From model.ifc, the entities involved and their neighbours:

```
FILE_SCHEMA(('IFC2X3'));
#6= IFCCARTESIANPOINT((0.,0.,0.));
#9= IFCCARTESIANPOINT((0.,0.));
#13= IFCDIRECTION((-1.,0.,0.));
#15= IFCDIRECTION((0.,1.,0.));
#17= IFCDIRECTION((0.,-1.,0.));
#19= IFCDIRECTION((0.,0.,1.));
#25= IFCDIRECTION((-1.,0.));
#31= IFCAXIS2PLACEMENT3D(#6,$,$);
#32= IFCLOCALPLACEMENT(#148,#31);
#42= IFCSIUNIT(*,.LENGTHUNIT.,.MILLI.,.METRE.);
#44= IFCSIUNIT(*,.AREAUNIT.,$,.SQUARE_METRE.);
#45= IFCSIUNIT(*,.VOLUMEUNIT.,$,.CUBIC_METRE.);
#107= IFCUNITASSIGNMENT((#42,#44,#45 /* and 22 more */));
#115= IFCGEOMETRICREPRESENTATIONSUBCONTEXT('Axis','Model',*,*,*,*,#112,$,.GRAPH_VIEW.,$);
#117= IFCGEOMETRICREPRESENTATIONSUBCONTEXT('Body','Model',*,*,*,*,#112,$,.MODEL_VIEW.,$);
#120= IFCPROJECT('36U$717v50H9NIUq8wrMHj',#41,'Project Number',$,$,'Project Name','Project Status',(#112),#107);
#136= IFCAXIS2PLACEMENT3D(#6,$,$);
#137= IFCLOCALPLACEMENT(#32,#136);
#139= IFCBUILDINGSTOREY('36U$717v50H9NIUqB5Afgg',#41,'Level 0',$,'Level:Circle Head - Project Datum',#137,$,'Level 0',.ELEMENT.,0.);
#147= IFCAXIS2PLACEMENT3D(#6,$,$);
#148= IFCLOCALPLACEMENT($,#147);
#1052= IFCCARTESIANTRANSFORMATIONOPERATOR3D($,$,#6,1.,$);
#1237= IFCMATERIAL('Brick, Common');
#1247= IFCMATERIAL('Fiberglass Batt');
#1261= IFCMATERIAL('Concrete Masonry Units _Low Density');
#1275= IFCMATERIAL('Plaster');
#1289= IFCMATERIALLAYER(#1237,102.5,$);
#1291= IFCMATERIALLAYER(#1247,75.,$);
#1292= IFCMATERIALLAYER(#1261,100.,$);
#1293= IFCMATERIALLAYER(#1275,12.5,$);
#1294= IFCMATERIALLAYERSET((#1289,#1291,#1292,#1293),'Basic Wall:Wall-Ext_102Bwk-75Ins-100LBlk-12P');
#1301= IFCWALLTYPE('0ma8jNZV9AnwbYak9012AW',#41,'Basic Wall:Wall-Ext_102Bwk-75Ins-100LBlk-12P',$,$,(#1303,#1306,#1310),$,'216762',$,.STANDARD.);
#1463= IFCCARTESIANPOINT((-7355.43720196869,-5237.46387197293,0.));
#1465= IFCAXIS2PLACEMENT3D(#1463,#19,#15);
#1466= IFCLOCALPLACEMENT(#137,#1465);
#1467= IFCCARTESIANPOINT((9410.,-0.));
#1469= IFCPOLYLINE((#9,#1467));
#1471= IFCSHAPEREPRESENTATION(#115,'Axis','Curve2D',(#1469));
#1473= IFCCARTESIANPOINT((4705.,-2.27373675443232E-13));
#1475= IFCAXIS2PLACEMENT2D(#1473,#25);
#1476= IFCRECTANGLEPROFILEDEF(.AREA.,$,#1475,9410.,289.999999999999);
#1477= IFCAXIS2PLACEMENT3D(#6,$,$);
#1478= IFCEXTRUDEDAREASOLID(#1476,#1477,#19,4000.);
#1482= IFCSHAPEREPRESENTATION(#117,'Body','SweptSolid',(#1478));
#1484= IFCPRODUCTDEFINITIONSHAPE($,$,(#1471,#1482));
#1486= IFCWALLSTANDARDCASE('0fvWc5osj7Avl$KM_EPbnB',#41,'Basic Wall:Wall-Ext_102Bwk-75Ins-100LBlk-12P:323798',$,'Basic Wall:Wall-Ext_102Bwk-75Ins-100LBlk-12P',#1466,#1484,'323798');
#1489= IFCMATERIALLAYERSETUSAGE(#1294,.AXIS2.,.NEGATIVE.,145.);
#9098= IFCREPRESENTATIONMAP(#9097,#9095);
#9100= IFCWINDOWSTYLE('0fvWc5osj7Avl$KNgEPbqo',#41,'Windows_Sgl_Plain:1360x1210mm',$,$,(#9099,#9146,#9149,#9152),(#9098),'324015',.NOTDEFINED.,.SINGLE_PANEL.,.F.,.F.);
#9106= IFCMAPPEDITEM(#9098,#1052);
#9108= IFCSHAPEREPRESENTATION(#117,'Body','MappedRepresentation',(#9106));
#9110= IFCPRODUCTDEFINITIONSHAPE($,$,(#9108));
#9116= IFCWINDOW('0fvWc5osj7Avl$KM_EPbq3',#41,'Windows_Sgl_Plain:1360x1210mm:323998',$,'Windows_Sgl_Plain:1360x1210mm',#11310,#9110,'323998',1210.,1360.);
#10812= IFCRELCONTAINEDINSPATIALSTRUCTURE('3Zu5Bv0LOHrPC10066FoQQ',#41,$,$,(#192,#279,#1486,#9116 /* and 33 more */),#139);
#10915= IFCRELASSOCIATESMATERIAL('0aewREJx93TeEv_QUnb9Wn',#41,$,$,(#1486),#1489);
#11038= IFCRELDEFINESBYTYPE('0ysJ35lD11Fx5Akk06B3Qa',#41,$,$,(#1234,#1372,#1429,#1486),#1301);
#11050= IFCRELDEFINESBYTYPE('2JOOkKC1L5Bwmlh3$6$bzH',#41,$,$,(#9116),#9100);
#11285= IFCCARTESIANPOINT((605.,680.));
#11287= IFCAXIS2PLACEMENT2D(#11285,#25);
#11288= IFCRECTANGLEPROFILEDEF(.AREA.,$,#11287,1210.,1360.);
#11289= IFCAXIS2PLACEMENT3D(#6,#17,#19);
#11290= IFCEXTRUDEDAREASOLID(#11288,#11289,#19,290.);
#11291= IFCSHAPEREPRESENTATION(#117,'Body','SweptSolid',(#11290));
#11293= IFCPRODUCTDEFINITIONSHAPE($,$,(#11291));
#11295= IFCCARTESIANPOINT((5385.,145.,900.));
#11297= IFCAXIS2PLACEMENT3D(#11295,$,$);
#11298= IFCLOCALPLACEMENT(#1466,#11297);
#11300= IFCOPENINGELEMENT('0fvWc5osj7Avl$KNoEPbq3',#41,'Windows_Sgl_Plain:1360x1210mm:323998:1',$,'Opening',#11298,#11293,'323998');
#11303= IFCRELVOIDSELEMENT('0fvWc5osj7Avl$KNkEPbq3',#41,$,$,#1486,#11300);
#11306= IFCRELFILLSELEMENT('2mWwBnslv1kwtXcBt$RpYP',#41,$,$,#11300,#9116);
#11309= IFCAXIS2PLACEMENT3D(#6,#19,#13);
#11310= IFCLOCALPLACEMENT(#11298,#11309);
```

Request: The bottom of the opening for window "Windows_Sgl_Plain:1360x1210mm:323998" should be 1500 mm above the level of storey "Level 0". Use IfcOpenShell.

```python
import numpy as np
import ifcopenshell
import ifcopenshell.api.geometry
import ifcopenshell.geom
import ifcopenshell.util.element
import ifcopenshell.util.placement
import ifcopenshell.util.shape
import ifcopenshell.util.unit

model = ifcopenshell.open("model.ifc")
unit_scale = ifcopenshell.util.unit.calculate_unit_scale(model)

window = model.by_id(9116)
opening = window.FillsVoids[0].RelatingOpeningElement
storey = ifcopenshell.util.element.get_container(window, ifc_class="IfcBuildingStorey")
level = ifcopenshell.util.placement.get_local_placement(storey.ObjectPlacement)[2, 3]

# The opening's origin need not be at the sill, so measure its lowest point.
shape = ifcopenshell.geom.create_shape(ifcopenshell.geom.settings(), opening)
bottom = ifcopenshell.util.shape.get_shape_bottom_elevation(shape, shape.geometry) / unit_scale
dz = level + 1.5 / unit_scale - bottom

shift = np.array([0.0, 0.0, dz])
# The window is placed relative to its opening, so it follows when the opening moves.
matrix = ifcopenshell.util.placement.get_local_placement(opening.ObjectPlacement)
matrix[:3, 3] += shift
ifcopenshell.api.geometry.edit_object_placement(
    model, product=opening, matrix=matrix, is_si=False, should_transform_children=True
)

print(f"moved by {dz * unit_scale:+.3f} m")

model.write("model_updated.ifc")
```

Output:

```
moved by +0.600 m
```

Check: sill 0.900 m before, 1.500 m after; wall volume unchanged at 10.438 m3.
